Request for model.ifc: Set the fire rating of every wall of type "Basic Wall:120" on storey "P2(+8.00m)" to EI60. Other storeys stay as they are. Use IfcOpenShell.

First a look at what the model holds.

```python
import ifcopenshell
import ifcopenshell.util.element

model = ifcopenshell.open("model.ifc")
print(model.schema)
storey = next(s for s in model.by_type("IfcBuildingStorey") if s.Name == "P2(+8.00m)")
walls = [e for e in ifcopenshell.util.element.get_decomposition(storey) if e.is_a("IfcWall")]
seen = {}
for e in walls:
    element_type = ifcopenshell.util.element.get_type(e)
    key = (element_type.Name if element_type != e and element_type else None, ifcopenshell.util.element.get_pset(e, "Pset_WallCommon", "FireRating"))
    seen[key] = seen.get(key, 0) + 1
for (name, value), count in sorted(seen.items(), key=str):
    print(count, "x", name, "|", value)
```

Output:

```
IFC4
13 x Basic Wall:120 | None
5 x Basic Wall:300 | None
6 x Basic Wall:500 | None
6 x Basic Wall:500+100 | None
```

```python
import ifcopenshell
import ifcopenshell.api.pset
import ifcopenshell.util.element

model = ifcopenshell.open("model.ifc")

storey = next(s for s in model.by_type("IfcBuildingStorey") if s.Name == "P2(+8.00m)")
walls = [e for e in ifcopenshell.util.element.get_decomposition(storey) if e.is_a("IfcWall")]

count = 0
for e in walls:
    element_type = ifcopenshell.util.element.get_type(e)
    if element_type in (None, e) or element_type.Name != "Basic Wall:120":
        continue
    # add_pset returns the element's existing set when there is one.
    pset = ifcopenshell.api.pset.add_pset(model, product=e, name="Pset_WallCommon")
    ifcopenshell.api.pset.edit_pset(model, pset=pset, properties={"FireRating": "EI60"})
    count += 1

print(count, "walls updated")

model.write("model_updated.ifc")
```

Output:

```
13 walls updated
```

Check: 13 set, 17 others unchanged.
